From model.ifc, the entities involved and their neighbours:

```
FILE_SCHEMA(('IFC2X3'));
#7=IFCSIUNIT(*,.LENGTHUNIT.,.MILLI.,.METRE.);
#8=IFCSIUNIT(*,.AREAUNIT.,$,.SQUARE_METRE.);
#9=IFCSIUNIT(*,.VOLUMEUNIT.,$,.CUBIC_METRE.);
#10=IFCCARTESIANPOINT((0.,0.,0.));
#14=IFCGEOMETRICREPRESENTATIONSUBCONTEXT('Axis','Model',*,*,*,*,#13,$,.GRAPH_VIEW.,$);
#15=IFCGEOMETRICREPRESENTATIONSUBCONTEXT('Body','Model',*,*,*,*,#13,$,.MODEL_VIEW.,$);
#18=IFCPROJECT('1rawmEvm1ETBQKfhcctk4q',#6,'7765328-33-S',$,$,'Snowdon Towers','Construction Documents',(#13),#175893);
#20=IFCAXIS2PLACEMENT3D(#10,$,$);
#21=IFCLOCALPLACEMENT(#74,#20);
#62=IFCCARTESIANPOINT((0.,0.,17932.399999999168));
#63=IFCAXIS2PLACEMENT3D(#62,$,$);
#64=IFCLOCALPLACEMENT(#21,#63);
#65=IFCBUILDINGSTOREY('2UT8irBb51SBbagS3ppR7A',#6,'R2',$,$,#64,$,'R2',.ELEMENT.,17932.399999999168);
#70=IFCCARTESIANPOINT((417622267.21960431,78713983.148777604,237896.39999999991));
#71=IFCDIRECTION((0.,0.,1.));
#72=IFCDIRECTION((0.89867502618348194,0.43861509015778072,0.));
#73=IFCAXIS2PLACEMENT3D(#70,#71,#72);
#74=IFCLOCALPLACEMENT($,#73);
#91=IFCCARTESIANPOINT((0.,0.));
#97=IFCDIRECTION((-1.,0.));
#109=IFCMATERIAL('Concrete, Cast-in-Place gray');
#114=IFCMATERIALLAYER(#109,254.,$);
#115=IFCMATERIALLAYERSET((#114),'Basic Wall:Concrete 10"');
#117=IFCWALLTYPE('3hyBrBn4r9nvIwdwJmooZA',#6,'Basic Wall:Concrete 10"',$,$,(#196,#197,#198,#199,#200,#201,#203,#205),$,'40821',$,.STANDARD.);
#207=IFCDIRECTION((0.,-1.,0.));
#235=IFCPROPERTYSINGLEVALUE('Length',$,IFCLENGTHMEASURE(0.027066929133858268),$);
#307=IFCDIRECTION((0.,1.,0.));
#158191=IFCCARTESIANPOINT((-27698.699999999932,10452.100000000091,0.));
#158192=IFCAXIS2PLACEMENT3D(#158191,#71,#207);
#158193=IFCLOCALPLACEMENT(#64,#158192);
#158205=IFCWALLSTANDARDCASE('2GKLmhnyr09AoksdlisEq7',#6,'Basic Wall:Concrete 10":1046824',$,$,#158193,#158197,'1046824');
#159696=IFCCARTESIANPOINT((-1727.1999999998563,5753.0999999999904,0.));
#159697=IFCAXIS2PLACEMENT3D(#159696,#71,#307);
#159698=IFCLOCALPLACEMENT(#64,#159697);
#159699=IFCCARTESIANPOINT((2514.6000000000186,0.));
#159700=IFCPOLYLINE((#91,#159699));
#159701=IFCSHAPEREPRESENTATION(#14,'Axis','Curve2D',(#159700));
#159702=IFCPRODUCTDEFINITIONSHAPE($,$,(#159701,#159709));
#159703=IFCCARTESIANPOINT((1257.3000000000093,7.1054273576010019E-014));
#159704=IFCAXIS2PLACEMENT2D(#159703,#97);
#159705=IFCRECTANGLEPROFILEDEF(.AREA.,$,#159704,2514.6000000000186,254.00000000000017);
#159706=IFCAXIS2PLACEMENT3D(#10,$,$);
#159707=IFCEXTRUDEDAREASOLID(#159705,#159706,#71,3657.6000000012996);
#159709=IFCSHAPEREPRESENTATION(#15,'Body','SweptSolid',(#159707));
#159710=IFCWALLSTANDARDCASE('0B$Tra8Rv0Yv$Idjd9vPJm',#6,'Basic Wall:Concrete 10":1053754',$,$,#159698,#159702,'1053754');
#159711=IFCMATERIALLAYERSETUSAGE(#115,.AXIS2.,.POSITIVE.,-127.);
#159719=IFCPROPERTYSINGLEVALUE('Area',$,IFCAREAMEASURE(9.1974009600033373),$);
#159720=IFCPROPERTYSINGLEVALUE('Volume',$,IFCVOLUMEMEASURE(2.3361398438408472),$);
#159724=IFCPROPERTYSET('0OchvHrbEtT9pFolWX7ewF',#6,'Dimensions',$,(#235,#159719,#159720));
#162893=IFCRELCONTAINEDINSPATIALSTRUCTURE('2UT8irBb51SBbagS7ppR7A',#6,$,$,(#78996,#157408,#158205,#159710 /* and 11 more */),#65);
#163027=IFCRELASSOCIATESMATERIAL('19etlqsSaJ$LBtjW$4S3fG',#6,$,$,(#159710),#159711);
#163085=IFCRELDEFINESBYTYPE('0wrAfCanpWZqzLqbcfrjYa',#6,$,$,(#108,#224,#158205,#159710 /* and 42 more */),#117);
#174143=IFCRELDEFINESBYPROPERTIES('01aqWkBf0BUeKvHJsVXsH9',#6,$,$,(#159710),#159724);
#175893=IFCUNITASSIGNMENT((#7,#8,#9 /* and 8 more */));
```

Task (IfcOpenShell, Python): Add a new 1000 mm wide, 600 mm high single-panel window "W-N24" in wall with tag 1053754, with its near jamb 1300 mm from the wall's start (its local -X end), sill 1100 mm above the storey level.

```python
import numpy as np
import ifcopenshell
import ifcopenshell.api.feature
import ifcopenshell.api.geometry
import ifcopenshell.api.pset
import ifcopenshell.api.root
import ifcopenshell.api.spatial
import ifcopenshell.api.type
import ifcopenshell.geom
import ifcopenshell.util.element
import ifcopenshell.util.placement
import ifcopenshell.util.representation
import ifcopenshell.util.shape
import ifcopenshell.util.unit

model = ifcopenshell.open("model.ifc")
unit_scale = ifcopenshell.util.unit.calculate_unit_scale(model)
area_scale = ifcopenshell.util.unit.calculate_unit_scale(model, "AREAUNIT")
volume_scale = ifcopenshell.util.unit.calculate_unit_scale(model, "VOLUMEUNIT")
settings = ifcopenshell.geom.settings()


def volume(element):
    """Net volume in cubic metres, openings subtracted."""
    shape = ifcopenshell.geom.create_shape(settings, element)
    return ifcopenshell.util.shape.get_volume(shape.geometry)


wall = model.by_guid("0B$Tra8Rv0Yv$Idjd9vPJm")
storey = ifcopenshell.util.element.get_container(wall, ifc_class="IfcBuildingStorey")
context = ifcopenshell.util.representation.get_context(model, "Model", "Body", "MODEL_VIEW")
before = volume(wall)

width, height, from_end, sill = 1, 0.6, 1.3, 1.1  # metres

# The wall runs along its own X axis, and the end named is its -X end.
wall_shape = ifcopenshell.geom.create_shape(settings, wall)
x, y, z = ifcopenshell.util.shape.get_vertices(wall_shape.geometry).T
start = x.min() + from_end
face, thickness = float(y.min()), float(y.max() - y.min())
wall_matrix = ifcopenshell.util.placement.get_local_placement(wall.ObjectPlacement)
level = ifcopenshell.util.placement.get_local_placement(storey.ObjectPlacement)[2, 3]


def in_wall(x, y):
    """Placement at x, y metres in the wall's axes, at sill height."""
    matrix = wall_matrix.copy()
    matrix[:, 3] = wall_matrix @ np.array([x / unit_scale, y / unit_scale, 0.0, 1.0])
    matrix[2, 3] = level + sill / unit_scale
    return matrix


# Opening: a box that overshoots both wall faces by 50 mm.
opening = ifcopenshell.api.root.create_entity(model, ifc_class="IfcOpeningElement")
box = ifcopenshell.api.geometry.add_wall_representation(
    model, context=context, length=width, height=height, thickness=thickness + 0.1
)
ifcopenshell.api.geometry.assign_representation(model, product=opening, representation=box)
ifcopenshell.api.geometry.edit_object_placement(model, product=opening, matrix=in_wall(start, face - 0.05), is_si=False)
ifcopenshell.api.feature.add_feature(model, feature=opening, element=wall)

window = ifcopenshell.api.root.create_entity(model, ifc_class="IfcWindow", name="W-N24")
window.OverallWidth, window.OverallHeight = width / unit_scale, height / unit_scale
body = ifcopenshell.api.geometry.add_window_representation(
    model,
    context=context,
    overall_width=window.OverallWidth,
    overall_height=window.OverallHeight,
    partition_type="SINGLE_PANEL",
)
ifcopenshell.api.geometry.assign_representation(model, product=window, representation=body)
ifcopenshell.api.spatial.assign_container(model, products=[window], relating_structure=storey)
fills = ifcopenshell.api.feature.add_filling(model, opening=opening, element=window)
fills.OwnerHistory = window.OwnerHistory  # required in IFC2X3

# IFC2X3 keeps the operation on the window style.
style = ifcopenshell.api.root.create_entity(model, ifc_class="IfcWindowStyle", name="W-N24")
style.OperationType, style.ConstructionType = "SINGLE_PANEL", "NOTDEFINED"
style.ParameterTakesPrecedence = style.Sizeable = False
ifcopenshell.api.type.assign_type(model, related_objects=[window], relating_type=style)

# Centre the window in the wall's thickness.
ifcopenshell.api.geometry.edit_object_placement(model, product=window, matrix=in_wall(start, face), is_si=False)
window_shape = ifcopenshell.geom.create_shape(settings, window)
depth = ifcopenshell.util.shape.get_vertices(window_shape.geometry)[:, 1]
offset = face + thickness / 2 - (depth.min() + depth.max()) / 2
ifcopenshell.api.geometry.edit_object_placement(model, product=window, matrix=in_wall(start, offset), is_si=False)

after = volume(wall)

# Update the wall's stored quantities.
pset = model.by_id(ifcopenshell.util.element.get_pset(wall, "Dimensions", should_inherit=False)["id"])
ifcopenshell.api.pset.edit_pset(model, pset=pset, properties={
    "Area": model.create_entity("IfcAreaMeasure", after / thickness / area_scale),
    "Volume": model.create_entity("IfcVolumeMeasure", after / volume_scale),
})

print(f"wall volume {before:.3f} -> {after:.3f} m3")

model.write("model_updated.ifc")
```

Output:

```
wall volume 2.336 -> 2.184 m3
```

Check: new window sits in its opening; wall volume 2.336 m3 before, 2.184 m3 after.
